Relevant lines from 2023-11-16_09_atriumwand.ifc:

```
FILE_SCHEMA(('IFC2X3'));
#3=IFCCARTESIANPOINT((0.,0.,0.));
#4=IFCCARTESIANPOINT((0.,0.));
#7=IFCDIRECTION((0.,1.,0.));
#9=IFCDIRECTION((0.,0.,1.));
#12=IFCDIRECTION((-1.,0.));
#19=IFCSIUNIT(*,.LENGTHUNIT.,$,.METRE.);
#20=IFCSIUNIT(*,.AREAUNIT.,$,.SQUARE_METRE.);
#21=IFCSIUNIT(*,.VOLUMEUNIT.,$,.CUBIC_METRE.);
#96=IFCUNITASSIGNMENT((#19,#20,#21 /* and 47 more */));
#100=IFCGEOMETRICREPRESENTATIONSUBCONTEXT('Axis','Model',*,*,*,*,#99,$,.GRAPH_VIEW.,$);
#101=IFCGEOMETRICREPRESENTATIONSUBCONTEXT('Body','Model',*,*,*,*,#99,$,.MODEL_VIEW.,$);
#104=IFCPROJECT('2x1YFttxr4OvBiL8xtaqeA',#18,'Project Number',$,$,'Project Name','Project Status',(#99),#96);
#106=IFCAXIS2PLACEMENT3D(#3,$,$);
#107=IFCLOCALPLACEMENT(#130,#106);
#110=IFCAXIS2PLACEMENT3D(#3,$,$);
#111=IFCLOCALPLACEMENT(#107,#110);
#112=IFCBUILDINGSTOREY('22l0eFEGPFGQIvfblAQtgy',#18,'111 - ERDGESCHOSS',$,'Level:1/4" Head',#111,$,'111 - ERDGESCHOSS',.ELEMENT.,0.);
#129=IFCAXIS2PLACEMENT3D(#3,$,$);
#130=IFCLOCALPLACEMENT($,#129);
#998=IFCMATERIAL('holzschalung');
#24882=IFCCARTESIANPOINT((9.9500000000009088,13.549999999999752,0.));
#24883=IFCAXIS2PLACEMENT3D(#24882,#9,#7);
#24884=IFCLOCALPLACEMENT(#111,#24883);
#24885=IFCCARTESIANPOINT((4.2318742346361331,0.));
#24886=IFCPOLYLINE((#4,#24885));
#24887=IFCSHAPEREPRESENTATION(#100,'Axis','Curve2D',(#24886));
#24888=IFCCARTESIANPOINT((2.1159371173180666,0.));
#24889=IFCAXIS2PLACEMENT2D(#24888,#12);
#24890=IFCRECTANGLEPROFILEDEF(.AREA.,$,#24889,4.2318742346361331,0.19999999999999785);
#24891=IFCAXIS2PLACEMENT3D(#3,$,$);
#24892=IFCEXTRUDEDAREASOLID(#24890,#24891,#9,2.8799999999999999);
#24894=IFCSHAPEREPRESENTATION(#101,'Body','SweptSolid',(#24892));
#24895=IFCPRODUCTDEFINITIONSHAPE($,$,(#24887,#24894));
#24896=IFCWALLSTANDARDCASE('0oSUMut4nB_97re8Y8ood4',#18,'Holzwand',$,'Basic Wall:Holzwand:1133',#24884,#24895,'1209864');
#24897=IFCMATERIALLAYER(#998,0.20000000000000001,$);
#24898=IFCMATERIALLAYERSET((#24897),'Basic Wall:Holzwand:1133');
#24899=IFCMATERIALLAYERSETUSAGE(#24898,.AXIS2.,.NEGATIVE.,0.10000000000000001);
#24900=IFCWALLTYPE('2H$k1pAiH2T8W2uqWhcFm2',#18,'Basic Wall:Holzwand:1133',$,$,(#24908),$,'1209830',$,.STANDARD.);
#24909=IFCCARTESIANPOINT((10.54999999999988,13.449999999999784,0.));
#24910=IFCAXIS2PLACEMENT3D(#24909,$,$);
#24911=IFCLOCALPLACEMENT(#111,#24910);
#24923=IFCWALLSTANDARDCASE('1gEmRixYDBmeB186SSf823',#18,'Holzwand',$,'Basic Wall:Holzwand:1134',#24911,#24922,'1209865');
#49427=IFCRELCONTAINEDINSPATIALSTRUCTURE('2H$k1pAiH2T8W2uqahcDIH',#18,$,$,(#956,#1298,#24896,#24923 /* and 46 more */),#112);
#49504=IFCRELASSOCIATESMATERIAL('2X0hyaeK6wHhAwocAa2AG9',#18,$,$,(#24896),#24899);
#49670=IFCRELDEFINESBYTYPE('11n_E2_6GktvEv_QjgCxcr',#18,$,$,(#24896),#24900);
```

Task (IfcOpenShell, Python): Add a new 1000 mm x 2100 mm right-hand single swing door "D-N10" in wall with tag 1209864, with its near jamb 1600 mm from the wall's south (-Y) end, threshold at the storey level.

```python
import numpy as np
import ifcopenshell
import ifcopenshell.api.feature
import ifcopenshell.api.geometry
import ifcopenshell.api.root
import ifcopenshell.api.spatial
import ifcopenshell.api.type
import ifcopenshell.geom
import ifcopenshell.util.element
import ifcopenshell.util.placement
import ifcopenshell.util.representation
import ifcopenshell.util.shape
import ifcopenshell.util.unit

model = ifcopenshell.open("2023-11-16_09_atriumwand.ifc")
unit_scale = ifcopenshell.util.unit.calculate_unit_scale(model)
settings = ifcopenshell.geom.settings()


def volume(element):
    """Net volume in cubic metres, openings subtracted."""
    shape = ifcopenshell.geom.create_shape(settings, element)
    return ifcopenshell.util.shape.get_volume(shape.geometry)


wall = model.by_id(24896)
storey = ifcopenshell.util.element.get_container(wall, ifc_class="IfcBuildingStorey")
context = ifcopenshell.util.representation.get_context(model, "Model", "Body", "MODEL_VIEW")
before = volume(wall)

width, height, from_end, sill = 1, 2.1, 1.6, 0.0  # metres

# The wall runs along its own X axis, and the end named is its -X end.
wall_shape = ifcopenshell.geom.create_shape(settings, wall)
x, y, z = ifcopenshell.util.shape.get_vertices(wall_shape.geometry).T
start = x.min() + from_end
face, thickness = float(y.min()), float(y.max() - y.min())
wall_matrix = ifcopenshell.util.placement.get_local_placement(wall.ObjectPlacement)
level = ifcopenshell.util.placement.get_local_placement(storey.ObjectPlacement)[2, 3]


def in_wall(x, y):
    """Placement at x, y metres in the wall's axes, at sill height."""
    matrix = wall_matrix.copy()
    matrix[:, 3] = wall_matrix @ np.array([x / unit_scale, y / unit_scale, 0.0, 1.0])
    matrix[2, 3] = level + sill / unit_scale
    return matrix


# Opening: a box that overshoots both wall faces by 50 mm.
opening = ifcopenshell.api.root.create_entity(model, ifc_class="IfcOpeningElement")
box = ifcopenshell.api.geometry.add_wall_representation(
    model, context=context, length=width, height=height, thickness=thickness + 0.1
)
ifcopenshell.api.geometry.assign_representation(model, product=opening, representation=box)
ifcopenshell.api.geometry.edit_object_placement(model, product=opening, matrix=in_wall(start, face - 0.05), is_si=False)
ifcopenshell.api.feature.add_feature(model, feature=opening, element=wall)

door = ifcopenshell.api.root.create_entity(model, ifc_class="IfcDoor", name="D-N10")
door.OverallWidth, door.OverallHeight = width / unit_scale, height / unit_scale
body = ifcopenshell.api.geometry.add_door_representation(
    model,
    context=context,
    overall_width=door.OverallWidth,
    overall_height=door.OverallHeight,
    operation_type="SINGLE_SWING_RIGHT",
    lining_properties={"LiningDepth": thickness / unit_scale, "ThresholdDepth": thickness / unit_scale},
)
ifcopenshell.api.geometry.assign_representation(model, product=door, representation=body)
ifcopenshell.api.spatial.assign_container(model, products=[door], relating_structure=storey)
fills = ifcopenshell.api.feature.add_filling(model, opening=opening, element=door)
fills.OwnerHistory = door.OwnerHistory  # required in IFC2X3

# IFC2X3 keeps the operation on the door style.
style = ifcopenshell.api.root.create_entity(model, ifc_class="IfcDoorStyle", name="D-N10")
style.OperationType, style.ConstructionType = "SINGLE_SWING_RIGHT", "NOTDEFINED"
style.ParameterTakesPrecedence = style.Sizeable = False
ifcopenshell.api.type.assign_type(model, related_objects=[door], relating_type=style)

# The lining spans the wall, so the door starts at the wall face.
ifcopenshell.api.geometry.edit_object_placement(model, product=door, matrix=in_wall(start, face), is_si=False)

after = volume(wall)

print(f"wall volume {before:.3f} -> {after:.3f} m3")

model.write("2023-11-16_09_atriumwand_v2.ifc")
```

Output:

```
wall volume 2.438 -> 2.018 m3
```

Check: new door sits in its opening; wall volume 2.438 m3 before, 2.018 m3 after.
